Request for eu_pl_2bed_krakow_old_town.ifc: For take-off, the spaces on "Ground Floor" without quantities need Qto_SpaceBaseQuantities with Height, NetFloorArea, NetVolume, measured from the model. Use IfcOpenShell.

First a look at what the model holds.

```python
import ifcopenshell
import ifcopenshell.util.element
import ifcopenshell.util.unit

model = ifcopenshell.open("eu_pl_2bed_krakow_old_town.ifc")
print(model.schema)
for unit_type in ("LENGTHUNIT", "AREAUNIT", "VOLUMEUNIT"):
    print(unit_type, ifcopenshell.util.unit.calculate_unit_scale(model, unit_type))
storey = next(s for s in model.by_type("IfcBuildingStorey") if s.Name == "Ground Floor")
spaces = [e for e in ifcopenshell.util.element.get_decomposition(storey) if e.is_a("IfcSpace")]
for e in sorted(spaces, key=lambda e: e.id()):
    print(e.id(), e.is_a(), e.Name, list(ifcopenshell.util.element.get_psets(e, qtos_only=True)), sep=" | ")
```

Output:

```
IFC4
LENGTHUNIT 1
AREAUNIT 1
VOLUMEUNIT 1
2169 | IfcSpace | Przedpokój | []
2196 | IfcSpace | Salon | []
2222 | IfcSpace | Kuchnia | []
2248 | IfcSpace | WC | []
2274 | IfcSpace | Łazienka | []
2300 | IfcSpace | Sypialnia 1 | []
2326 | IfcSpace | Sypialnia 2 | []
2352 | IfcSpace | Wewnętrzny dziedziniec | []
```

```python
import ifcopenshell
import ifcopenshell.api.pset
import ifcopenshell.geom
import ifcopenshell.util.element
import ifcopenshell.util.shape
import ifcopenshell.util.unit

model = ifcopenshell.open("eu_pl_2bed_krakow_old_town.ifc")
unit_scale = ifcopenshell.util.unit.calculate_unit_scale(model)
area_scale = ifcopenshell.util.unit.calculate_unit_scale(model, "AREAUNIT")
volume_scale = ifcopenshell.util.unit.calculate_unit_scale(model, "VOLUMEUNIT")
settings = ifcopenshell.geom.settings()

storey = next(s for s in model.by_type("IfcBuildingStorey") if s.Name == "Ground Floor")
spaces = [e for e in ifcopenshell.util.element.get_decomposition(storey) if e.is_a("IfcSpace")]

for e in sorted(spaces, key=lambda e: e.id()):
    if ifcopenshell.util.element.get_psets(e, qtos_only=True, should_inherit=False):
        continue
    # Geometry comes back in metres, in the element's own axes.
    shape = ifcopenshell.geom.create_shape(settings, e)
    values = {
        "Height": ifcopenshell.util.shape.get_z(shape.geometry) / unit_scale,
        "NetFloorArea": ifcopenshell.util.shape.get_footprint_area(shape.geometry) / area_scale,
        "NetVolume": ifcopenshell.util.shape.get_volume(shape.geometry) / volume_scale,
    }
    qto = ifcopenshell.api.pset.add_qto(model, product=e, name="Qto_SpaceBaseQuantities")
    ifcopenshell.api.pset.edit_qto(model, qto=qto, properties=values)
    print(e.id(), {k: round(v, 3) for k, v in values.items()})

model.write("eu_pl_2bed_krakow_old_town-out.ifc")
```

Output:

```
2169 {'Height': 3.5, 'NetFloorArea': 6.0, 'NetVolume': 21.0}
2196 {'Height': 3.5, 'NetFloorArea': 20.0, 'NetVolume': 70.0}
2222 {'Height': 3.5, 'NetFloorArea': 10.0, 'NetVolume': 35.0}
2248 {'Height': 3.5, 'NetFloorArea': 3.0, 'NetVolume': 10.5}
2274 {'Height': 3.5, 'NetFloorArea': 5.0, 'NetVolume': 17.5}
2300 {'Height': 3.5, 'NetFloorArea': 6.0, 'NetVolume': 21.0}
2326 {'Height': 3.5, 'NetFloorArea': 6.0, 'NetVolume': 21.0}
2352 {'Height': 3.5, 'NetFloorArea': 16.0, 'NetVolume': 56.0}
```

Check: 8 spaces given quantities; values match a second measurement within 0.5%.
